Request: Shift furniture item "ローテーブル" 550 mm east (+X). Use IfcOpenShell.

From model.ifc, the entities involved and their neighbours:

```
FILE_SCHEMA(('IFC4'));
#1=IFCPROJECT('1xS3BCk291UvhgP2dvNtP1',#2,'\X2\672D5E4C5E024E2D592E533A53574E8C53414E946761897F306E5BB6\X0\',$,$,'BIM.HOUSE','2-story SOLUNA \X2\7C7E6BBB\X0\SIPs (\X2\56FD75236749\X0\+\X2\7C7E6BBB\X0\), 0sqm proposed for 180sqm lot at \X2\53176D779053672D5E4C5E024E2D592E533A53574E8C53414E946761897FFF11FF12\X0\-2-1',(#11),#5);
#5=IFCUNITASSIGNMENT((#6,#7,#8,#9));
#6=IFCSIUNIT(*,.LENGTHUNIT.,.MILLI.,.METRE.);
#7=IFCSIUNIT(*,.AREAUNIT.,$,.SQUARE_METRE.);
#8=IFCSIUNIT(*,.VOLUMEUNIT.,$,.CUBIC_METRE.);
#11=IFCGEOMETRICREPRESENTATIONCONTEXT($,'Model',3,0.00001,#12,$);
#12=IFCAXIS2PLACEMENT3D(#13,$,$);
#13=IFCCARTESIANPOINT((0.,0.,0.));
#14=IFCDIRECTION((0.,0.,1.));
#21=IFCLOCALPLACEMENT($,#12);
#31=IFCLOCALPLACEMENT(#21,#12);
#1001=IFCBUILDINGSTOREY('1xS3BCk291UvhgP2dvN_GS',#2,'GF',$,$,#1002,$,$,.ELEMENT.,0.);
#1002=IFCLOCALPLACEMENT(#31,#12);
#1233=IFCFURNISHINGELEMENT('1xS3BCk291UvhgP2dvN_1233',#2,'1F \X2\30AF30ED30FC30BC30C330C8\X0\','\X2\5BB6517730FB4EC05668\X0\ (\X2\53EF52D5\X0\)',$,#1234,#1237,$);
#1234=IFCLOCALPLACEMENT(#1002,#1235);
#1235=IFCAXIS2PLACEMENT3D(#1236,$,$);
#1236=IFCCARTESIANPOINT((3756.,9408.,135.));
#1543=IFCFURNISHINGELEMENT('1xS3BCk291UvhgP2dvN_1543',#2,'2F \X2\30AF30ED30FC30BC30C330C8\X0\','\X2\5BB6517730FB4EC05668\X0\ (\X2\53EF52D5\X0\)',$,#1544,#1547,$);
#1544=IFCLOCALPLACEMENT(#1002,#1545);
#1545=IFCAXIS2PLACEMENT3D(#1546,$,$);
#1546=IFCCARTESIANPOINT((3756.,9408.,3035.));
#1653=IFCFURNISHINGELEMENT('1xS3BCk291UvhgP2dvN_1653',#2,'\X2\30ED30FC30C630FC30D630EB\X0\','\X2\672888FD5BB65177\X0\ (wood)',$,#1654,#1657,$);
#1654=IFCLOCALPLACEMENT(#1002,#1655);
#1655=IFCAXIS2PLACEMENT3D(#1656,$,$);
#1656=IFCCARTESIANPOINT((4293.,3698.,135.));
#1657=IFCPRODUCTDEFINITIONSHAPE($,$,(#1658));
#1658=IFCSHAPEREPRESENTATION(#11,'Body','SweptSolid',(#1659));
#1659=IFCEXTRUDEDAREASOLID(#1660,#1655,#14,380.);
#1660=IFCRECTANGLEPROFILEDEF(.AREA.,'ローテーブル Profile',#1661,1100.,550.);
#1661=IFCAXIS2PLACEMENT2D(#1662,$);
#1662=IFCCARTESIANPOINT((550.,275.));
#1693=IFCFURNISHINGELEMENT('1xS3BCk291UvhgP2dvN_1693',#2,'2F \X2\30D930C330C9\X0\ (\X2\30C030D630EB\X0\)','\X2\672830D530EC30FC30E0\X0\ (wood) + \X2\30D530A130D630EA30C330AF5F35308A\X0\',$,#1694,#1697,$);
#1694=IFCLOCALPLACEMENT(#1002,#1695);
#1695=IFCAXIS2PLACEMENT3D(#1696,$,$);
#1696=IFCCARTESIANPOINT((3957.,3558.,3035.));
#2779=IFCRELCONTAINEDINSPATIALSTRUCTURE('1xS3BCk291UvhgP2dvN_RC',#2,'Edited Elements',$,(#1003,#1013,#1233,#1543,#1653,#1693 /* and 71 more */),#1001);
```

```python
import ifcopenshell
import ifcopenshell.api.geometry
import ifcopenshell.util.placement
import ifcopenshell.util.unit

model = ifcopenshell.open("model.ifc")
unit_scale = ifcopenshell.util.unit.calculate_unit_scale(model)

item = model.by_id(1653)
matrix = ifcopenshell.util.placement.get_local_placement(item.ObjectPlacement)
matrix[0, 3] += 0.55 / unit_scale
ifcopenshell.api.geometry.edit_object_placement(model, product=item, matrix=matrix, is_si=False)

print(ifcopenshell.util.placement.get_local_placement(item.ObjectPlacement).round(3) + 0.0)

model.write("model_v2.ifc")
```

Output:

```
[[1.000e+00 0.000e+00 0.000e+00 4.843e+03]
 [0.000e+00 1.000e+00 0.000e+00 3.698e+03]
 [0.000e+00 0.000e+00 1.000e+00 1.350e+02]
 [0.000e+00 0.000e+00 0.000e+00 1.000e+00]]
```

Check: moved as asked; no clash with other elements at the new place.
